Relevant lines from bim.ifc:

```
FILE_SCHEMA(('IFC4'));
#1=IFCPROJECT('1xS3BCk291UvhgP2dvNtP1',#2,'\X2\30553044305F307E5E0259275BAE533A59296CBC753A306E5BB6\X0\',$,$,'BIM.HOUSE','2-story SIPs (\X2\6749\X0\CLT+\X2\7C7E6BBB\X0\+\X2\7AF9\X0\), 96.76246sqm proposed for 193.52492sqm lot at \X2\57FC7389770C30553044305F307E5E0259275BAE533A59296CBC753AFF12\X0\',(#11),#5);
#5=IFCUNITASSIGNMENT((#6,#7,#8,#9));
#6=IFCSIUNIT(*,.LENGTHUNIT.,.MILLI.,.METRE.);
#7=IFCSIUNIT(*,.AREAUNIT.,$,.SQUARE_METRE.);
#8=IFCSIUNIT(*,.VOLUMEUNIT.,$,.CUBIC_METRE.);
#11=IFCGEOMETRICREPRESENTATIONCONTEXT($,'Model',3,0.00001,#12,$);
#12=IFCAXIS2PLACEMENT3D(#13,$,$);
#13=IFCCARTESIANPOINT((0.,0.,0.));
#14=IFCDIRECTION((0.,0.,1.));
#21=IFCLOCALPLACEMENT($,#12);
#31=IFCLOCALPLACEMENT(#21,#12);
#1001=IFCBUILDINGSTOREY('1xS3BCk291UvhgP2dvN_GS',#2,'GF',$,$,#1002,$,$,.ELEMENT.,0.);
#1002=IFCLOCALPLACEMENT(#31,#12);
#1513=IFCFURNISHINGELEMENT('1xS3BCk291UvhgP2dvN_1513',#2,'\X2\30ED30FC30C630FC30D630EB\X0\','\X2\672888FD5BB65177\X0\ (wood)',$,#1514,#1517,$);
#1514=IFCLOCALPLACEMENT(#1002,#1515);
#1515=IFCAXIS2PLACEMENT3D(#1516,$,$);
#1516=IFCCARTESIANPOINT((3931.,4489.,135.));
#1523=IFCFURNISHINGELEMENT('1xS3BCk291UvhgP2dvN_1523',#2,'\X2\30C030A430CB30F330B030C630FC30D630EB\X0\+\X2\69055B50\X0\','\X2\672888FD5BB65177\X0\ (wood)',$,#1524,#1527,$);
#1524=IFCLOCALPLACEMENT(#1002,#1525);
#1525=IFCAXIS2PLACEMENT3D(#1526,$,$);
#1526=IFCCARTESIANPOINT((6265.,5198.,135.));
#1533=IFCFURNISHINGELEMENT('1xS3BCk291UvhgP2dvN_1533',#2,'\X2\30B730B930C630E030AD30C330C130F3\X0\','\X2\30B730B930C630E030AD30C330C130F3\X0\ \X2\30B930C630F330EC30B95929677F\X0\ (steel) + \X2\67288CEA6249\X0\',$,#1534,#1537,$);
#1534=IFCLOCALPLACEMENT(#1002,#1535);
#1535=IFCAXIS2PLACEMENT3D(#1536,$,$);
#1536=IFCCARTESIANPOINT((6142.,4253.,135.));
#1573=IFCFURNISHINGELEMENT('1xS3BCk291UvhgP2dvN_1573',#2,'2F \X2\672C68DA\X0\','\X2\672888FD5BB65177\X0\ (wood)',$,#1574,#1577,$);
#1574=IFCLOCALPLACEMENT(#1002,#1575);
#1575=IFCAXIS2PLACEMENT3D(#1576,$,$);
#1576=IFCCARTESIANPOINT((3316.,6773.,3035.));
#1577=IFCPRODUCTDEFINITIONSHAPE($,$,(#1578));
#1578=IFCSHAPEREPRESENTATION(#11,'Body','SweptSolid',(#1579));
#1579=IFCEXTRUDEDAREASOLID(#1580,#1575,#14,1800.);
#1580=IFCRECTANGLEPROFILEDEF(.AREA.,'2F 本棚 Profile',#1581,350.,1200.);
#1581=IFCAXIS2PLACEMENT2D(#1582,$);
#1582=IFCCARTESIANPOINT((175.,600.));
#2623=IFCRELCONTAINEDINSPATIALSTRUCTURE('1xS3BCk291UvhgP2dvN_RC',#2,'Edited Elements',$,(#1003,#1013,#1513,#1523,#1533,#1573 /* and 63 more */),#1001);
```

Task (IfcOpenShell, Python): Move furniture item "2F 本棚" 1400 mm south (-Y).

```python
import ifcopenshell
import ifcopenshell.api.geometry
import ifcopenshell.util.placement
import ifcopenshell.util.unit

model = ifcopenshell.open("bim.ifc")
unit_scale = ifcopenshell.util.unit.calculate_unit_scale(model)

item = model.by_guid("1xS3BCk291UvhgP2dvN_1573")
matrix = ifcopenshell.util.placement.get_local_placement(item.ObjectPlacement)
matrix[1, 3] -= 1.4 / unit_scale
ifcopenshell.api.geometry.edit_object_placement(model, product=item, matrix=matrix, is_si=False)

print(ifcopenshell.util.placement.get_local_placement(item.ObjectPlacement).round(3) + 0.0)

model.write("bim-out.ifc")
```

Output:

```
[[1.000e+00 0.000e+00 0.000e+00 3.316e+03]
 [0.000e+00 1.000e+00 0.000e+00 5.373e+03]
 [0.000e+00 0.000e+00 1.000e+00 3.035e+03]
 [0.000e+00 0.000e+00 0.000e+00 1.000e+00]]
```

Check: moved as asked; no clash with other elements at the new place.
